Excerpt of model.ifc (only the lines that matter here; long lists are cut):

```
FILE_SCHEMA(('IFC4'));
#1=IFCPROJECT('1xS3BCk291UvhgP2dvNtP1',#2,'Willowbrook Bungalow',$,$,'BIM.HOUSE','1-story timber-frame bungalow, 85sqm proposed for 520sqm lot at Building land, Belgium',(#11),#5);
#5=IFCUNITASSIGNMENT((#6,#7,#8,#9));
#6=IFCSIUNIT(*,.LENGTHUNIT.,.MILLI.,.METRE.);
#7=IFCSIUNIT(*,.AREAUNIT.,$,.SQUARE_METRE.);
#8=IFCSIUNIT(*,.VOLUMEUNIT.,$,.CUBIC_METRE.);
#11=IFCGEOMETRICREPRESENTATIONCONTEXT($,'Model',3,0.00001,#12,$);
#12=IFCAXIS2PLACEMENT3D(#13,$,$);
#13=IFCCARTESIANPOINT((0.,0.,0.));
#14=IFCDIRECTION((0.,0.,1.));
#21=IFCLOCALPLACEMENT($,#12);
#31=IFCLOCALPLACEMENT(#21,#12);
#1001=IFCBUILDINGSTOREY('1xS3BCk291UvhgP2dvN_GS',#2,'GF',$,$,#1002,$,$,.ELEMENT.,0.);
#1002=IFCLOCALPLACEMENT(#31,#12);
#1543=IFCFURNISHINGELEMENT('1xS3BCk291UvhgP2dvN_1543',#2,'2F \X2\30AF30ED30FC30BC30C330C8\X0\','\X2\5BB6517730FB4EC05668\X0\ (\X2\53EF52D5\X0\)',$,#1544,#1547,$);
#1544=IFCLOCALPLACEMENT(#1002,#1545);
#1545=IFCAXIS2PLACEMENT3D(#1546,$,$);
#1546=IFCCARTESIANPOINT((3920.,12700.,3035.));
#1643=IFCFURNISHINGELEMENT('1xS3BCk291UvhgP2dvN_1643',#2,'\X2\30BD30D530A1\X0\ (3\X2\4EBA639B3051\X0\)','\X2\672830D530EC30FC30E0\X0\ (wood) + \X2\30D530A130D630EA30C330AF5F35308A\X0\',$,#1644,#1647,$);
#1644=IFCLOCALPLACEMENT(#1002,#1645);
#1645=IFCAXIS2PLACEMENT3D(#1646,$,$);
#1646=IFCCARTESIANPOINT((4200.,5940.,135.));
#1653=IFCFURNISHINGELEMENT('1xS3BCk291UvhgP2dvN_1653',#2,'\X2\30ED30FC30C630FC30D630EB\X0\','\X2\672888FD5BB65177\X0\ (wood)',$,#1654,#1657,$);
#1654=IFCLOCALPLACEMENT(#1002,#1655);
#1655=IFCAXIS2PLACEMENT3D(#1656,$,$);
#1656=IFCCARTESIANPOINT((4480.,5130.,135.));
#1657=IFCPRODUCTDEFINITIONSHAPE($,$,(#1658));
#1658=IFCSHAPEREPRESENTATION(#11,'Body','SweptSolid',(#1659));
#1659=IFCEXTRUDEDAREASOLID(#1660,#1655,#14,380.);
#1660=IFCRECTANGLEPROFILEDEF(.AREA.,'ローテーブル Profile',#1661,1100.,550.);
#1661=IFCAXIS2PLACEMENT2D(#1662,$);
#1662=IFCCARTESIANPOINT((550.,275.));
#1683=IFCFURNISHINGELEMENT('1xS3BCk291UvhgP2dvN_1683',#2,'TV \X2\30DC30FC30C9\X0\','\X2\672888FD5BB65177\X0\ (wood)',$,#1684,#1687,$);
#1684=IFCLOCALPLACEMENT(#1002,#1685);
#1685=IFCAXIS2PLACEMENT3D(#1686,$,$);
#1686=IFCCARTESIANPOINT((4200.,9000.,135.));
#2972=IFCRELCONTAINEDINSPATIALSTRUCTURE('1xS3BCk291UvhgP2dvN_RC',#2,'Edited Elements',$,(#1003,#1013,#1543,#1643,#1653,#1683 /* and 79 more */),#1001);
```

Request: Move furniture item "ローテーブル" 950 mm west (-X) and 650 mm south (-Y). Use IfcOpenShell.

```python
import ifcopenshell
import ifcopenshell.api.geometry
import ifcopenshell.util.placement
import ifcopenshell.util.unit

model = ifcopenshell.open("model.ifc")
unit_scale = ifcopenshell.util.unit.calculate_unit_scale(model)

item = model.by_guid("1xS3BCk291UvhgP2dvN_1653")
matrix = ifcopenshell.util.placement.get_local_placement(item.ObjectPlacement)
matrix[0, 3] -= 0.95 / unit_scale
matrix[1, 3] -= 0.65 / unit_scale
ifcopenshell.api.geometry.edit_object_placement(model, product=item, matrix=matrix, is_si=False)

print(ifcopenshell.util.placement.get_local_placement(item.ObjectPlacement).round(3) + 0.0)

model.write("model_updated.ifc")
```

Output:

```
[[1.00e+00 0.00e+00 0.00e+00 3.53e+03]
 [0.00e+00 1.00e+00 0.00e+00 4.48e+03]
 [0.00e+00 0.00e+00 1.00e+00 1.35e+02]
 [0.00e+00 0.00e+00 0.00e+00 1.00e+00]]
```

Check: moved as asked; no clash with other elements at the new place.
